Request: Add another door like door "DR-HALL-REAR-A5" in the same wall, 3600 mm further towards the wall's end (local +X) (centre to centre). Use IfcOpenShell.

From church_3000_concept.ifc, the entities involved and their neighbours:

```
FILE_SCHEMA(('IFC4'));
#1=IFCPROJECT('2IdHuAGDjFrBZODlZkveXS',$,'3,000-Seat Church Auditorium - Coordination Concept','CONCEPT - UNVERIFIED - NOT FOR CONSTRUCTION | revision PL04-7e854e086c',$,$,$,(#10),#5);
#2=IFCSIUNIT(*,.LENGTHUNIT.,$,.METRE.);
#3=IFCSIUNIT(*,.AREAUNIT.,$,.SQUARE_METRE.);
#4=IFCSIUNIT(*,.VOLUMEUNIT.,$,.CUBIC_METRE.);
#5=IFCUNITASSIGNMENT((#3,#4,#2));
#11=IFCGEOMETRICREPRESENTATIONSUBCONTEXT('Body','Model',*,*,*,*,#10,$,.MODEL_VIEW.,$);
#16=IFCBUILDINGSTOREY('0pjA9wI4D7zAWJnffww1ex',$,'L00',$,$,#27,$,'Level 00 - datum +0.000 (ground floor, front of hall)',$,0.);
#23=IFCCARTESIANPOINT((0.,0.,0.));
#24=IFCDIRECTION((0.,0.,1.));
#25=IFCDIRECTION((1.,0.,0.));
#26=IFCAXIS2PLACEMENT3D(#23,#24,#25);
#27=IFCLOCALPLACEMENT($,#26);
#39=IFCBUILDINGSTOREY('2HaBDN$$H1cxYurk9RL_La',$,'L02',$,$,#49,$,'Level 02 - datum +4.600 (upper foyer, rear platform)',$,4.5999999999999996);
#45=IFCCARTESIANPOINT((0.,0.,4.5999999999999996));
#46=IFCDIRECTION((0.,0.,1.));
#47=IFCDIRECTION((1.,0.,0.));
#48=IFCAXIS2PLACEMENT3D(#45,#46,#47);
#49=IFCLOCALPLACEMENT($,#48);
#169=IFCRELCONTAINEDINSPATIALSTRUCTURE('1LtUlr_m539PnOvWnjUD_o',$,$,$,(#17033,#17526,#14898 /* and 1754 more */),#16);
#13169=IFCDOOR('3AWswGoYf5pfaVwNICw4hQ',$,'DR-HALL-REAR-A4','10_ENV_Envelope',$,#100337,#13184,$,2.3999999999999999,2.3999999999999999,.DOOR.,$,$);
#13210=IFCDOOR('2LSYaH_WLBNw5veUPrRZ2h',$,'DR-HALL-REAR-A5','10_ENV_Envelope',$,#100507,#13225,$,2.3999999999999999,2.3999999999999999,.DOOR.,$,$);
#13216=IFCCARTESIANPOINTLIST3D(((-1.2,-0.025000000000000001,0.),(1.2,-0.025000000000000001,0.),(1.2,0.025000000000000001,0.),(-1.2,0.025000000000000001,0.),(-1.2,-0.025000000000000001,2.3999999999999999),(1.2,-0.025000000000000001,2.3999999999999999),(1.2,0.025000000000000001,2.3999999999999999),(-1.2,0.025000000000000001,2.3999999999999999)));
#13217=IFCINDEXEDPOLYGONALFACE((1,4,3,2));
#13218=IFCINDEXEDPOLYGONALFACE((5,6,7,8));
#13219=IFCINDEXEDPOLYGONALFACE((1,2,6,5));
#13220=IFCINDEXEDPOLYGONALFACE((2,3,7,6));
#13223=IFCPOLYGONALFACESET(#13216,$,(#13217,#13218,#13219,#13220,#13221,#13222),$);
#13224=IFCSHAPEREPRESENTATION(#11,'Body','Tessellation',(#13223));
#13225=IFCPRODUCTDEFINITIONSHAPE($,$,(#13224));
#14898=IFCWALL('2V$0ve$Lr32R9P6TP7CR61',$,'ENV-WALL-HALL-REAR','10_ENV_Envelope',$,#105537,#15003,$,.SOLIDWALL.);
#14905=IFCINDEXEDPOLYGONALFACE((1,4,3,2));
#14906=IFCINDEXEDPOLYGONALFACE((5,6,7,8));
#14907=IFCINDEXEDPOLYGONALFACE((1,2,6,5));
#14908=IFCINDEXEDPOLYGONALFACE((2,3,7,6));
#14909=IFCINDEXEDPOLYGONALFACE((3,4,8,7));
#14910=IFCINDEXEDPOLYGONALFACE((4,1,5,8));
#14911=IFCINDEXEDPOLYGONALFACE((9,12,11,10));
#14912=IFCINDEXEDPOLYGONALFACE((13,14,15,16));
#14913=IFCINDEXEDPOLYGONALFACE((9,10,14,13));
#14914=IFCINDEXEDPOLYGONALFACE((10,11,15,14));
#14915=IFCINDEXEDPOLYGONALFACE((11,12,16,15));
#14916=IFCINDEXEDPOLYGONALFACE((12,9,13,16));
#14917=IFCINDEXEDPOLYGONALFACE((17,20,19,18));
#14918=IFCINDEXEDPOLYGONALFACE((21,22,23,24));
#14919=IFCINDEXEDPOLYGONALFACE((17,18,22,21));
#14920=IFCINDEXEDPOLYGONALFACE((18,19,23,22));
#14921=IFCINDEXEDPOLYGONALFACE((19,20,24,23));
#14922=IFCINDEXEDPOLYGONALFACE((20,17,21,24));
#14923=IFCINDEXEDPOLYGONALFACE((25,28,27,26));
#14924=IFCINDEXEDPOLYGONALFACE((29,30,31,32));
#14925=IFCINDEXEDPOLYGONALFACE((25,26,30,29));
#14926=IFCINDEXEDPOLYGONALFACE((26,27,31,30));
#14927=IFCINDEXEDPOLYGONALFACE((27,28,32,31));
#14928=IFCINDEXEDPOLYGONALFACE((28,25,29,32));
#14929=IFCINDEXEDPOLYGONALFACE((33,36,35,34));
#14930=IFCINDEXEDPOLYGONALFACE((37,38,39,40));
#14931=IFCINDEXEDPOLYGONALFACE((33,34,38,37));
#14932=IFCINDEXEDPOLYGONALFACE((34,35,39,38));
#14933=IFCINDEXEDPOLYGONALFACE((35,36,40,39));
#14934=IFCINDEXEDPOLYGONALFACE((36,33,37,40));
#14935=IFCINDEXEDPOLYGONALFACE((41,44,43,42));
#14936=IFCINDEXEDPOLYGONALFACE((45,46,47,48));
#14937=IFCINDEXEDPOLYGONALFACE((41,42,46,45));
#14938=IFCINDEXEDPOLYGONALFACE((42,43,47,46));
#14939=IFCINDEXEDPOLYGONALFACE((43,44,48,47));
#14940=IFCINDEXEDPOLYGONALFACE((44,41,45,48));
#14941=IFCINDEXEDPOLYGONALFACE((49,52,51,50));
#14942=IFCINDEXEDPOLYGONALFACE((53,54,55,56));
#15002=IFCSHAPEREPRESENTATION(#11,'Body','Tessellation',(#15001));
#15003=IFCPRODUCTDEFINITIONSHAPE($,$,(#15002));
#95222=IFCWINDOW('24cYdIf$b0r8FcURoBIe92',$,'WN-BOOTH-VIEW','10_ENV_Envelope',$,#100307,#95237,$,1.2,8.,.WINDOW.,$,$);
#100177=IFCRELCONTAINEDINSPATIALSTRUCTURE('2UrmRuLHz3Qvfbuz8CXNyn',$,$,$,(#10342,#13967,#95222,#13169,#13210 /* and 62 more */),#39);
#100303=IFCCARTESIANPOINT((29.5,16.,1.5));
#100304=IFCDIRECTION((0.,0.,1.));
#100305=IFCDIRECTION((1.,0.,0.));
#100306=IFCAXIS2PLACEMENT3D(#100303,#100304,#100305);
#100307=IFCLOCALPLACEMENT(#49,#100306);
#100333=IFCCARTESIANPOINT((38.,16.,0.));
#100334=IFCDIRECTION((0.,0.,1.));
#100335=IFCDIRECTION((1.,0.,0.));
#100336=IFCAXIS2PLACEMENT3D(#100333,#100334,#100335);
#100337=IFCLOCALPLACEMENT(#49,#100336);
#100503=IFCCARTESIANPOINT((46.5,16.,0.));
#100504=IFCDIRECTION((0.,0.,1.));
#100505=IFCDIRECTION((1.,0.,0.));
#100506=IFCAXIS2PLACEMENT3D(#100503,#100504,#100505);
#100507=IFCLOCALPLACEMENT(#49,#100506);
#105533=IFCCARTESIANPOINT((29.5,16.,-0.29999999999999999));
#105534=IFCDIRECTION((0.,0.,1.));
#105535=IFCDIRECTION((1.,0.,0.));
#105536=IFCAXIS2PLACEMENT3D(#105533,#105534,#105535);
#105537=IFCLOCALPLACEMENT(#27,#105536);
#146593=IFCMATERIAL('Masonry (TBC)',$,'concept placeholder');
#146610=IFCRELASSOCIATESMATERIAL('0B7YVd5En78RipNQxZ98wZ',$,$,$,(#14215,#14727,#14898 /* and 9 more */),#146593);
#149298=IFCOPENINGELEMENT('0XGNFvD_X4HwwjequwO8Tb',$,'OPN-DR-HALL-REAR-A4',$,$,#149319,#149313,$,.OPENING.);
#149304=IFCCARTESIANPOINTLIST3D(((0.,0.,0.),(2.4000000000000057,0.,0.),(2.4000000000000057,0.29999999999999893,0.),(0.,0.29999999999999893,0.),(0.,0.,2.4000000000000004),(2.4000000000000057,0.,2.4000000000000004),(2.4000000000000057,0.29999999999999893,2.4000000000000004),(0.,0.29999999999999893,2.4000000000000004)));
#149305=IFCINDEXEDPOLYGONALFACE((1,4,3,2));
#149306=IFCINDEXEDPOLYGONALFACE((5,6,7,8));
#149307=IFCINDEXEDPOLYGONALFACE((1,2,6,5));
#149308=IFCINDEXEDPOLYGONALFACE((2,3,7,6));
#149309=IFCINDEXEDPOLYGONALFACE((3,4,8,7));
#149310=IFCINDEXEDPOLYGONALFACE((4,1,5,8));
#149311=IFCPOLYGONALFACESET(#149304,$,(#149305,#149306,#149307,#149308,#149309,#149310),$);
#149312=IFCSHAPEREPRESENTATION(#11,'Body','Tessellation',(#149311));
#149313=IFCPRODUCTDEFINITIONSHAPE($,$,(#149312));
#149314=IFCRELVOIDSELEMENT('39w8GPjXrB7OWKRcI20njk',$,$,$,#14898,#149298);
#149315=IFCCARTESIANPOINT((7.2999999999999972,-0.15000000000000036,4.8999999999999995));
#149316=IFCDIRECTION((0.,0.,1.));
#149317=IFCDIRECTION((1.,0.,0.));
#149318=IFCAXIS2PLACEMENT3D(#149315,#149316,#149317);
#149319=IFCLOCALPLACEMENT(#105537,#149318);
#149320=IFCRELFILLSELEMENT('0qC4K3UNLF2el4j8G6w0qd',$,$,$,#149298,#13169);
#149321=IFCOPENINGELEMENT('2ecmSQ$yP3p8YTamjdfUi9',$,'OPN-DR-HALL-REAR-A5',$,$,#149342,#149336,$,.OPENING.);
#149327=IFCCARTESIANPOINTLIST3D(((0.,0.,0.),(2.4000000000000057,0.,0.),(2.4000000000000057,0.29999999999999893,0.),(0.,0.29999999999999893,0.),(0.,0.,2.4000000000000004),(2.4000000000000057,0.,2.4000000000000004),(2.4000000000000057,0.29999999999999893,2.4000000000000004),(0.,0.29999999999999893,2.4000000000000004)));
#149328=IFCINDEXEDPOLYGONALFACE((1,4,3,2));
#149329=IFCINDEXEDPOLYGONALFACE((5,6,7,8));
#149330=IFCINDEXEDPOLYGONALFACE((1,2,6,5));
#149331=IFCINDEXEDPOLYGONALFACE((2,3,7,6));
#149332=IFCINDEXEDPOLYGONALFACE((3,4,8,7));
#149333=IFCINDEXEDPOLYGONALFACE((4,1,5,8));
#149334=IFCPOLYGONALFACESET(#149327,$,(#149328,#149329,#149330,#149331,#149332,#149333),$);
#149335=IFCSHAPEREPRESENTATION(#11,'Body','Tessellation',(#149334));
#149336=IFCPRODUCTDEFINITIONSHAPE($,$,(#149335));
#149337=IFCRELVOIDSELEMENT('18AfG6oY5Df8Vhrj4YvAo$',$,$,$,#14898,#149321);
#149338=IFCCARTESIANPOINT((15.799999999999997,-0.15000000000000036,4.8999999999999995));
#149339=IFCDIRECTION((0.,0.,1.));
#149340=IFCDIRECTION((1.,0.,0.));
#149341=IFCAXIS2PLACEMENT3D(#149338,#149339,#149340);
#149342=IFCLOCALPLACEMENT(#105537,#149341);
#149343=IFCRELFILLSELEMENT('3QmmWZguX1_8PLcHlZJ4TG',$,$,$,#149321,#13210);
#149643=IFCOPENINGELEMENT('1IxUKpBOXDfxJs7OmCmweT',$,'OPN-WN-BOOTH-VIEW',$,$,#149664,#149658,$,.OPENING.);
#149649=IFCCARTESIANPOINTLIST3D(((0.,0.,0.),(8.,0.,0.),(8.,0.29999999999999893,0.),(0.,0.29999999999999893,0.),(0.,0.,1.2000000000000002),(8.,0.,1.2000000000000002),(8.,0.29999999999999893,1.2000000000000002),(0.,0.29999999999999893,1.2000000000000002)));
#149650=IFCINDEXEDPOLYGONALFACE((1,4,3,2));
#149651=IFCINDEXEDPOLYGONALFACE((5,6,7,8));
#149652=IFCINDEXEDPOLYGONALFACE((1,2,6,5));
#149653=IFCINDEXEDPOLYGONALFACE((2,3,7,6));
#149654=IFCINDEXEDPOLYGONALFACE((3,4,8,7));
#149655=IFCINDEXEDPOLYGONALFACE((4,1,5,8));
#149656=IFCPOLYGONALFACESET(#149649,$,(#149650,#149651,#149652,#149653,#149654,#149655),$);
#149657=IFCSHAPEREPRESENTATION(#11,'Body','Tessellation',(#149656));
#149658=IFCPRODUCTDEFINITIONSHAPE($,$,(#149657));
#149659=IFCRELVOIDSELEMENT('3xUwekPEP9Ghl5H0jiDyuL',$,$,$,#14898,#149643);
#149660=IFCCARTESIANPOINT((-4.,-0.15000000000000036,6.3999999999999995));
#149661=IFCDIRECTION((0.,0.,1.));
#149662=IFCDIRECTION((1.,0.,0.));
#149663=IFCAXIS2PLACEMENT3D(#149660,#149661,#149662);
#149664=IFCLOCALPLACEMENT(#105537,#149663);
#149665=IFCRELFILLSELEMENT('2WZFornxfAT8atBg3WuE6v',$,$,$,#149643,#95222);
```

```python
import ifcopenshell
import ifcopenshell.api.feature
import ifcopenshell.api.geometry
import ifcopenshell.api.root
import ifcopenshell.geom
import ifcopenshell.util.element
import ifcopenshell.util.placement
import ifcopenshell.util.shape
import ifcopenshell.util.unit

model = ifcopenshell.open("church_3000_concept.ifc")
unit_scale = ifcopenshell.util.unit.calculate_unit_scale(model)
settings = ifcopenshell.geom.settings()


def volume(element):
    """Net volume in cubic metres, openings subtracted."""
    shape = ifcopenshell.geom.create_shape(settings, element)
    return ifcopenshell.util.shape.get_volume(shape.geometry)


door = model.by_guid("2LSYaH_WLBNw5veUPrRZ2h")
opening = door.FillsVoids[0].RelatingOpeningElement
wall = opening.VoidsElements[0].RelatingBuildingElement
before = volume(wall)
shift = ifcopenshell.util.placement.get_local_placement(wall.ObjectPlacement)[:3, 0] * 3.6 / unit_scale

# copy_class copies the void relationship, type, container and properties, but no geometry.
new_opening = ifcopenshell.api.root.copy_class(model, product=opening)
new_opening.Representation = ifcopenshell.util.element.copy_deep(
    model, opening.Representation, exclude=["IfcGeometricRepresentationContext", "IfcRepresentationMap"]
)
new_door = ifcopenshell.api.root.copy_class(model, product=door)
new_door.Representation = ifcopenshell.util.element.copy_deep(
    model, door.Representation, exclude=["IfcGeometricRepresentationContext", "IfcRepresentationMap"]
)
ifcopenshell.api.feature.add_filling(model, opening=new_opening, element=new_door)

for old, new in ((opening, new_opening), (door, new_door)):
    matrix = ifcopenshell.util.placement.get_local_placement(old.ObjectPlacement)
    matrix[:3, 3] += shift
    ifcopenshell.api.geometry.edit_object_placement(model, product=new, matrix=matrix, is_si=False)

after = volume(wall)

print(f"wall volume {before:.3f} -> {after:.3f} m3")

model.write("church_3000_concept_updated.ifc")
```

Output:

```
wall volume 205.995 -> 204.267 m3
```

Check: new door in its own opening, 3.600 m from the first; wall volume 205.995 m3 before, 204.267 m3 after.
